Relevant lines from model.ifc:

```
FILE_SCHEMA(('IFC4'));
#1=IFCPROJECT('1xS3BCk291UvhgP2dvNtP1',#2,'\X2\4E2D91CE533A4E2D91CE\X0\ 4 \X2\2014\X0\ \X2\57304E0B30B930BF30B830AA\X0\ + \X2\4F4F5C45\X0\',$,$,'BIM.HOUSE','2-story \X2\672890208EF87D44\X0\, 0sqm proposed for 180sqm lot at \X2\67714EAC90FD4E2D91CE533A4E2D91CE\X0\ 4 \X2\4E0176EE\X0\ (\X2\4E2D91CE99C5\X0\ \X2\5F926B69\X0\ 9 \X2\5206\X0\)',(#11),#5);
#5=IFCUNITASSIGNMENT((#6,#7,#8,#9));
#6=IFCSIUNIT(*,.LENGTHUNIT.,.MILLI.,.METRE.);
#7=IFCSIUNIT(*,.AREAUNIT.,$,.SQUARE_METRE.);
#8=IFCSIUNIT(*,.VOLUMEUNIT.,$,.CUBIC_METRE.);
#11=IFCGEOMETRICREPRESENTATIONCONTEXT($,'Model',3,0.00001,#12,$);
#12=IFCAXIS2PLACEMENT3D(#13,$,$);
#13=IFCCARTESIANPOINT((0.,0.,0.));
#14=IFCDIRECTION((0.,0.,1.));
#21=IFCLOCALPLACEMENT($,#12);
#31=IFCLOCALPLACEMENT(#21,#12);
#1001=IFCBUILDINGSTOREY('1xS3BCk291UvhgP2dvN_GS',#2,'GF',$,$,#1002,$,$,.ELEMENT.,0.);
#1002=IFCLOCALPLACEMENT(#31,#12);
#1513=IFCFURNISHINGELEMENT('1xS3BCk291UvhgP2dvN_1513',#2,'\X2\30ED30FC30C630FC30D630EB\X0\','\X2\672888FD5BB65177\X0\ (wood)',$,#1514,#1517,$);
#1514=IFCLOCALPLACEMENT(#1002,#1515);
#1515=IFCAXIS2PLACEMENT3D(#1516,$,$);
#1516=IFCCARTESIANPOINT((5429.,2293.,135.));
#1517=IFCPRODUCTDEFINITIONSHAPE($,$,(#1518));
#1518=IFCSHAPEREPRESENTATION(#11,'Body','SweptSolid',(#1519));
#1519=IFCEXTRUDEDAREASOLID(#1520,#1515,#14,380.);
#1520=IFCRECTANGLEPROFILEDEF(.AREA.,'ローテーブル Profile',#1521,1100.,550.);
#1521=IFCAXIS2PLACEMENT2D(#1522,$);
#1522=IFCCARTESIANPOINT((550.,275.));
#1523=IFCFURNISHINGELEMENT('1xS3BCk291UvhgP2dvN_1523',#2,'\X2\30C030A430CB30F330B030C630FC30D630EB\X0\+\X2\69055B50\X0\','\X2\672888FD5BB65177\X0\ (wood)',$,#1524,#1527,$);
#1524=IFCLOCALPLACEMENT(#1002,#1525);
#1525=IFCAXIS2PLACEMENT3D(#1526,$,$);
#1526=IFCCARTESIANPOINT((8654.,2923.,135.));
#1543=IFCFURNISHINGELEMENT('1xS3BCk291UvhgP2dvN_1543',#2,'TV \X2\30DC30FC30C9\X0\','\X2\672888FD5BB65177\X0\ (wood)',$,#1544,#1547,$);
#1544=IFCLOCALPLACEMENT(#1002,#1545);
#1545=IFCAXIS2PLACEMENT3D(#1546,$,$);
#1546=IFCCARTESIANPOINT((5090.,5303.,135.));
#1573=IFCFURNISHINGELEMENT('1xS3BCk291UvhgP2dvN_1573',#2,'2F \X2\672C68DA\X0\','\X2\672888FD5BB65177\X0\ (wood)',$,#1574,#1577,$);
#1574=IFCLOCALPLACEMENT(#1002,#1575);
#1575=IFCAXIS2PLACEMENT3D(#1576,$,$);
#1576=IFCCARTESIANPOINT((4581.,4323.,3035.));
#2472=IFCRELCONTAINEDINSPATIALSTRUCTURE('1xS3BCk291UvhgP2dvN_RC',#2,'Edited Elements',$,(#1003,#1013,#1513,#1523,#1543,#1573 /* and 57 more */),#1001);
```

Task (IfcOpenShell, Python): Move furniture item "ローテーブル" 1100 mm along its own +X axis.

```python
import ifcopenshell
import ifcopenshell.api.geometry
import ifcopenshell.util.placement
import ifcopenshell.util.unit

model = ifcopenshell.open("model.ifc")
unit_scale = ifcopenshell.util.unit.calculate_unit_scale(model)

item = model.by_id(1513)
matrix = ifcopenshell.util.placement.get_local_placement(item.ObjectPlacement)
matrix[:3, 3] += matrix[:3, 0] * 1.1 / unit_scale
ifcopenshell.api.geometry.edit_object_placement(model, product=item, matrix=matrix, is_si=False)

print(ifcopenshell.util.placement.get_local_placement(item.ObjectPlacement).round(3) + 0.0)

model.write("model_edited.ifc")
```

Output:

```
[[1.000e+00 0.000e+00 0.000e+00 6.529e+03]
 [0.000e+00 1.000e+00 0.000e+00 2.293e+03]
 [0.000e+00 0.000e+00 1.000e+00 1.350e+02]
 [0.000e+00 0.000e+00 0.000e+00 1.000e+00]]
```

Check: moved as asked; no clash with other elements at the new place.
